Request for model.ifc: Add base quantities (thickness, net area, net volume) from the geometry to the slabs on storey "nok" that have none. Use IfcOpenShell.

First a look at what the model holds.

```python
import ifcopenshell
import ifcopenshell.util.element
import ifcopenshell.util.unit

model = ifcopenshell.open("model.ifc")
print(model.schema)
for unit_type in ("LENGTHUNIT", "AREAUNIT", "VOLUMEUNIT"):
    print(unit_type, ifcopenshell.util.unit.calculate_unit_scale(model, unit_type))
storey = next(s for s in model.by_type("IfcBuildingStorey") if s.Name == "nok")
slabs = [e for e in ifcopenshell.util.element.get_decomposition(storey) if e.is_a("IfcSlab")]
for e in sorted(slabs, key=lambda e: e.id()):
    print(e.id(), e.is_a(), e.Name, list(ifcopenshell.util.element.get_psets(e, qtos_only=True)), sep=" | ")
```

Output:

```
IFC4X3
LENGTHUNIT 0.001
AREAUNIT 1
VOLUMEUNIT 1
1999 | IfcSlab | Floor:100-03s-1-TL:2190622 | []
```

```python
import ifcopenshell
import ifcopenshell.api.pset
import ifcopenshell.geom
import ifcopenshell.util.element
import ifcopenshell.util.shape
import ifcopenshell.util.unit

model = ifcopenshell.open("model.ifc")
unit_scale = ifcopenshell.util.unit.calculate_unit_scale(model)
area_scale = ifcopenshell.util.unit.calculate_unit_scale(model, "AREAUNIT")
volume_scale = ifcopenshell.util.unit.calculate_unit_scale(model, "VOLUMEUNIT")
settings = ifcopenshell.geom.settings()

storey = next(s for s in model.by_type("IfcBuildingStorey") if s.Name == "nok")
slabs = [e for e in ifcopenshell.util.element.get_decomposition(storey) if e.is_a("IfcSlab")]

for e in sorted(slabs, key=lambda e: e.id()):
    if ifcopenshell.util.element.get_psets(e, qtos_only=True, should_inherit=False):
        continue
    # Geometry comes back in metres, in the element's own axes.
    shape = ifcopenshell.geom.create_shape(settings, e)
    values = {
        "Width": ifcopenshell.util.shape.get_z(shape.geometry) / unit_scale,
        "NetArea": ifcopenshell.util.shape.get_footprint_area(shape.geometry) / area_scale,
        "NetVolume": ifcopenshell.util.shape.get_volume(shape.geometry) / volume_scale,
    }
    qto = ifcopenshell.api.pset.add_qto(model, product=e, name="Qto_SlabBaseQuantities")
    ifcopenshell.api.pset.edit_qto(model, qto=qto, properties=values)
    print(e.id(), {k: round(v, 3) for k, v in values.items()})

model.write("model_edited.ifc")
```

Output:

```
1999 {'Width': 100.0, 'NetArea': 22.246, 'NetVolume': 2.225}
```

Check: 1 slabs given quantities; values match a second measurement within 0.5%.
